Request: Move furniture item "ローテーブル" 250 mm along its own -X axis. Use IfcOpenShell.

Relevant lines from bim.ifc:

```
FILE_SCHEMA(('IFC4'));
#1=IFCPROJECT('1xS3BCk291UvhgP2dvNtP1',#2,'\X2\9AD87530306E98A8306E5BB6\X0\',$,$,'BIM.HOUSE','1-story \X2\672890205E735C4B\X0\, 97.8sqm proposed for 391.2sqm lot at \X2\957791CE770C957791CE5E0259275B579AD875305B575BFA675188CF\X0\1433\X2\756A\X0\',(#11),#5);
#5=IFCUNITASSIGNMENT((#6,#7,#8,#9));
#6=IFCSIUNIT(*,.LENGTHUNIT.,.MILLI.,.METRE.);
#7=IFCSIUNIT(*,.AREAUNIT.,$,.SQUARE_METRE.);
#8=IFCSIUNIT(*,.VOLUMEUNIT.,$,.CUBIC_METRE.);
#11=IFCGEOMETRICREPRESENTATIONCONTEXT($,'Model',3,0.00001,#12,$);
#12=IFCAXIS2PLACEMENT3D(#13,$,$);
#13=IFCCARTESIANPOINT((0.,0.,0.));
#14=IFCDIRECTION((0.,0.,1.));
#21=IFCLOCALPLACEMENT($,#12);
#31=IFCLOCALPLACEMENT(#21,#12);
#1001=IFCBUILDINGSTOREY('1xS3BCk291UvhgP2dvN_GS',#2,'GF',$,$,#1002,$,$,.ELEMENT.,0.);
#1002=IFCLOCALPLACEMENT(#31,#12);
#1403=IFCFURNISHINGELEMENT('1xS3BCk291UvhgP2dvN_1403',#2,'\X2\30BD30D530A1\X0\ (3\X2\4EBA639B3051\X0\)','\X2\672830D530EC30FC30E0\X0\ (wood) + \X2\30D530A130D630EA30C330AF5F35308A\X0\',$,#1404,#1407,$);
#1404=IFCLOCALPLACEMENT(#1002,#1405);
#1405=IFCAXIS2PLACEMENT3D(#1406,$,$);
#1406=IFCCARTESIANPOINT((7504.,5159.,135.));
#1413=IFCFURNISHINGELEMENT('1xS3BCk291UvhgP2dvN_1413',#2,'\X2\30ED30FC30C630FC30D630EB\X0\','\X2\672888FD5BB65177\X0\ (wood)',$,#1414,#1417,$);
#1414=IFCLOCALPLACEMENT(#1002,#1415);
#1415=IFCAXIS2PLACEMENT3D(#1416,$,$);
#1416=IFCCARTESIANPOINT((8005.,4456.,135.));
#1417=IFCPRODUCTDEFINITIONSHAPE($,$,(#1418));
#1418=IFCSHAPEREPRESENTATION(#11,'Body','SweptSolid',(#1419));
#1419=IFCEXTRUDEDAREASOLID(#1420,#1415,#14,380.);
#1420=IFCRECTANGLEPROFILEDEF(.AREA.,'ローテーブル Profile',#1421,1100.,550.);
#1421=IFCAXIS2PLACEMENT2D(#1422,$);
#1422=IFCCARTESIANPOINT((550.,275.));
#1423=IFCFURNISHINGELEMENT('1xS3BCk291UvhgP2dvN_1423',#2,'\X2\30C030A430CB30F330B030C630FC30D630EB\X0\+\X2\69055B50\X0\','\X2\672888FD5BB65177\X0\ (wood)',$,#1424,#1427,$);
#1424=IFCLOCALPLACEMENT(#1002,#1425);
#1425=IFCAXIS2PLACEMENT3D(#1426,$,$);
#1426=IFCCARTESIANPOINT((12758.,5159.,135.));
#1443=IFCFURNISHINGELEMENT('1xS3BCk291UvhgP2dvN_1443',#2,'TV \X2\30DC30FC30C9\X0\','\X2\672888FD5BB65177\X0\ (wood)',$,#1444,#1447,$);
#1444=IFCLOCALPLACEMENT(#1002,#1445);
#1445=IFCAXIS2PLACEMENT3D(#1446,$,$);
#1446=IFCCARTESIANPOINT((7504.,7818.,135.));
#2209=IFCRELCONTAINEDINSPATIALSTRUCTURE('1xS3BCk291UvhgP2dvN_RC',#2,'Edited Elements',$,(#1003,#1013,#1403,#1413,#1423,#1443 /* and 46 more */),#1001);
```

```python
import ifcopenshell
import ifcopenshell.api.geometry
import ifcopenshell.util.placement

model = ifcopenshell.open("bim.ifc")

item = model.by_guid("1xS3BCk291UvhgP2dvN_1413")
matrix = ifcopenshell.util.placement.get_local_placement(item.ObjectPlacement)
matrix[:3, 3] -= matrix[:3, 0] * 250.0
ifcopenshell.api.geometry.edit_object_placement(model, product=item, matrix=matrix, is_si=False)

print(ifcopenshell.util.placement.get_local_placement(item.ObjectPlacement).round(3) + 0.0)

model.write("bim_v2.ifc")
```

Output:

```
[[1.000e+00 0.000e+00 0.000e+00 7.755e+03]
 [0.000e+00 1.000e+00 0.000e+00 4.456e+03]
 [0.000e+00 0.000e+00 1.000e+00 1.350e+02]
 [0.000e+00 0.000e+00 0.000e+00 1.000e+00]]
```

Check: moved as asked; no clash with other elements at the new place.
